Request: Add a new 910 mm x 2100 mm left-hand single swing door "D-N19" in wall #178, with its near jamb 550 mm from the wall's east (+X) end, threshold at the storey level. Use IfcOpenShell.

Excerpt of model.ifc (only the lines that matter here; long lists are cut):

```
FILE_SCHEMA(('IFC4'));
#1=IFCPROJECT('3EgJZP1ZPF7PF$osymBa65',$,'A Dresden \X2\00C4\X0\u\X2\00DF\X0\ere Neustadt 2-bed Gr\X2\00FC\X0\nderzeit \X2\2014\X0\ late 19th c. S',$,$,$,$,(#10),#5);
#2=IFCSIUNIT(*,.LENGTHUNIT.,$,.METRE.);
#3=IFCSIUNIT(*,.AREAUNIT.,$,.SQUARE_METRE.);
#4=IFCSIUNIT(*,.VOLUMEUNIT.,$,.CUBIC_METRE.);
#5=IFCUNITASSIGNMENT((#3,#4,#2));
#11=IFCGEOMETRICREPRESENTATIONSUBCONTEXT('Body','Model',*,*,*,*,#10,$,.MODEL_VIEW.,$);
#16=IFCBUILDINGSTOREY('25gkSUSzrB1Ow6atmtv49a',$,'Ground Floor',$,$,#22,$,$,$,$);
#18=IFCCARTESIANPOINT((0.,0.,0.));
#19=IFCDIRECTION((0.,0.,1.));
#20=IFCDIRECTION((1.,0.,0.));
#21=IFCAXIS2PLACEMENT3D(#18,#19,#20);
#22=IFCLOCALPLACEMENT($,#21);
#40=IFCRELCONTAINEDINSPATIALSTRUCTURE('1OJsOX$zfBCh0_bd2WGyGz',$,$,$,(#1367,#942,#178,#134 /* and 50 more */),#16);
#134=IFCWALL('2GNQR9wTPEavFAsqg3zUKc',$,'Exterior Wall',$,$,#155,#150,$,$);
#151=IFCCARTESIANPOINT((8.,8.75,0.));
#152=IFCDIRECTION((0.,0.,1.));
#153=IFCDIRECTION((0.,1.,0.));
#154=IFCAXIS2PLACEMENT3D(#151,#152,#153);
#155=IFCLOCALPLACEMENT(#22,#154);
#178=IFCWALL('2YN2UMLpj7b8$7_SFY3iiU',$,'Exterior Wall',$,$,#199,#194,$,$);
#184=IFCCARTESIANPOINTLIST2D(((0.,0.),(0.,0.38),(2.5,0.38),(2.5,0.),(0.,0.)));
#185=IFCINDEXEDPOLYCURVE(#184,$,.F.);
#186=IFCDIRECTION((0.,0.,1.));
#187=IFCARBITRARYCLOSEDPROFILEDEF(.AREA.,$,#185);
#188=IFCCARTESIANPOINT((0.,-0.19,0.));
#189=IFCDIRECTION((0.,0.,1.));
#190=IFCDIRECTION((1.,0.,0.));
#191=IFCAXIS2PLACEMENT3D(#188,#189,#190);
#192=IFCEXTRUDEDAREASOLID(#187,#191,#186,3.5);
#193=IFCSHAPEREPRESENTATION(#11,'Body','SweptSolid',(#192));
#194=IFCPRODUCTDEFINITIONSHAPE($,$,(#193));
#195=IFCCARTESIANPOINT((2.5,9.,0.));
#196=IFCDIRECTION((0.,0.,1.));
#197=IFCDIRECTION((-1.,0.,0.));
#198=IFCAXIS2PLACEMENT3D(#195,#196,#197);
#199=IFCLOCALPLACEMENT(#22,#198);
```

```python
import numpy as np
import ifcopenshell
import ifcopenshell.api.feature
import ifcopenshell.api.geometry
import ifcopenshell.api.root
import ifcopenshell.api.spatial
import ifcopenshell.geom
import ifcopenshell.util.element
import ifcopenshell.util.placement
import ifcopenshell.util.representation
import ifcopenshell.util.shape
import ifcopenshell.util.unit

model = ifcopenshell.open("model.ifc")
unit_scale = ifcopenshell.util.unit.calculate_unit_scale(model)
settings = ifcopenshell.geom.settings()


def volume(element):
    """Net volume in cubic metres, openings subtracted."""
    shape = ifcopenshell.geom.create_shape(settings, element)
    return ifcopenshell.util.shape.get_volume(shape.geometry)


wall = model.by_guid("2YN2UMLpj7b8$7_SFY3iiU")
storey = ifcopenshell.util.element.get_container(wall, ifc_class="IfcBuildingStorey")
context = ifcopenshell.util.representation.get_context(model, "Model", "Body", "MODEL_VIEW")
before = volume(wall)

width, height, from_end, sill = 0.91, 2.1, 0.55, 0.0  # metres

# The wall runs along its own X axis, and the end named is its -X end.
wall_shape = ifcopenshell.geom.create_shape(settings, wall)
x, y, z = ifcopenshell.util.shape.get_vertices(wall_shape.geometry).T
start = x.min() + from_end
face, thickness = float(y.min()), float(y.max() - y.min())
wall_matrix = ifcopenshell.util.placement.get_local_placement(wall.ObjectPlacement)
level = ifcopenshell.util.placement.get_local_placement(storey.ObjectPlacement)[2, 3]


def in_wall(x, y):
    """Placement at x, y metres in the wall's axes, at sill height."""
    matrix = wall_matrix.copy()
    matrix[:, 3] = wall_matrix @ np.array([x / unit_scale, y / unit_scale, 0.0, 1.0])
    matrix[2, 3] = level + sill / unit_scale
    return matrix


# Opening: a box that overshoots both wall faces by 50 mm.
opening = ifcopenshell.api.root.create_entity(model, ifc_class="IfcOpeningElement", predefined_type="OPENING")
box = ifcopenshell.api.geometry.add_wall_representation(
    model, context=context, length=width, height=height, thickness=thickness + 0.1
)
ifcopenshell.api.geometry.assign_representation(model, product=opening, representation=box)
ifcopenshell.api.geometry.edit_object_placement(model, product=opening, matrix=in_wall(start, face - 0.05), is_si=False)
ifcopenshell.api.feature.add_feature(model, feature=opening, element=wall)

door = ifcopenshell.api.root.create_entity(model, ifc_class="IfcDoor", name="D-N19", predefined_type="DOOR")
door.OverallWidth, door.OverallHeight = width / unit_scale, height / unit_scale
door.OperationType = "SINGLE_SWING_LEFT"
body = ifcopenshell.api.geometry.add_door_representation(
    model,
    context=context,
    overall_width=door.OverallWidth,
    overall_height=door.OverallHeight,
    operation_type="SINGLE_SWING_LEFT",
    lining_properties={"LiningDepth": thickness / unit_scale, "ThresholdDepth": thickness / unit_scale},
)
ifcopenshell.api.geometry.assign_representation(model, product=door, representation=body)
ifcopenshell.api.spatial.assign_container(model, products=[door], relating_structure=storey)
ifcopenshell.api.feature.add_filling(model, opening=opening, element=door)

# The lining spans the wall, so the door starts at the wall face.
ifcopenshell.api.geometry.edit_object_placement(model, product=door, matrix=in_wall(start, face), is_si=False)

after = volume(wall)

print(f"wall volume {before:.3f} -> {after:.3f} m3")

model.write("model-out.ifc")
```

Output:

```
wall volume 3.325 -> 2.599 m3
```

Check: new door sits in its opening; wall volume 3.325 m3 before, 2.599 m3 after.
